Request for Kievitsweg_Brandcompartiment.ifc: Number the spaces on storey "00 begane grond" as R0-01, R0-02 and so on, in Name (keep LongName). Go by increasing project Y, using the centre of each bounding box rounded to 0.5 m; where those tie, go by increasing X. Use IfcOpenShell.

First a look at what the model holds.

```python
import ifcopenshell
import ifcopenshell.util.element
import ifcopenshell.util.placement

model = ifcopenshell.open("Kievitsweg_Brandcompartiment.ifc")
print(model.schema)
storey = next(s for s in model.by_type("IfcBuildingStorey") if s.Name == "00 begane grond")
spaces = [e for e in ifcopenshell.util.element.get_decomposition(storey) if e.is_a("IfcSpace")]
for e in sorted(spaces, key=lambda e: e.id()):
    origin = ifcopenshell.util.placement.get_local_placement(e.ObjectPlacement)[:3, 3]
    print(e.id(), e.Name, e.LongName, origin.round(2) + 0.0, sep=" | ")
```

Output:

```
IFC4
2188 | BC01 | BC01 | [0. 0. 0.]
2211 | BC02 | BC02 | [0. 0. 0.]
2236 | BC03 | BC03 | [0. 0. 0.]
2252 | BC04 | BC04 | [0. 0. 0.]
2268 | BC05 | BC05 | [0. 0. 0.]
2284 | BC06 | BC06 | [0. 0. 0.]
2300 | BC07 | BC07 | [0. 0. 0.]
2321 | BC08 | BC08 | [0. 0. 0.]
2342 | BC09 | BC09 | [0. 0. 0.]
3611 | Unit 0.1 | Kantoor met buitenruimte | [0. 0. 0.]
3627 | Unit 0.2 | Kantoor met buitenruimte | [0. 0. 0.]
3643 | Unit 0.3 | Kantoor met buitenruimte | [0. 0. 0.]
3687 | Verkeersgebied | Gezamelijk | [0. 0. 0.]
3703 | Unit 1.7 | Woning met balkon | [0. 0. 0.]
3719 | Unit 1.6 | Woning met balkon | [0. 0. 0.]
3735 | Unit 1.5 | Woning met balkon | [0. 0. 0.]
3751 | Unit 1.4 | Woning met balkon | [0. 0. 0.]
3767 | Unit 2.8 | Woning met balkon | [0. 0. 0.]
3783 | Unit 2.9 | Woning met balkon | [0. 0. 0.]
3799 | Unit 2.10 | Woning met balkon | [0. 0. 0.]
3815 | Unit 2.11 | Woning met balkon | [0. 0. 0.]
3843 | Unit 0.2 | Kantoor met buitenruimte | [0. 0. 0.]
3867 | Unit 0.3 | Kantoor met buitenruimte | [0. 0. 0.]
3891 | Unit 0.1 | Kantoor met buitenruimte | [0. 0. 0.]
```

```python
import ifcopenshell
import ifcopenshell.geom
import ifcopenshell.util.element
import ifcopenshell.util.shape

model = ifcopenshell.open("Kievitsweg_Brandcompartiment.ifc")
settings = ifcopenshell.geom.settings()
settings.set("use-world-coords", True)


def centre(element):
    shape = ifcopenshell.geom.create_shape(settings, element)
    return ifcopenshell.util.shape.get_bbox_centroid(shape.geometry)


storey = next(s for s in model.by_type("IfcBuildingStorey") if s.Name == "00 begane grond")
spaces = [e for e in ifcopenshell.util.element.get_decomposition(storey) if e.is_a("IfcSpace")]

# Insertion points can sit at a corner or the storey origin, so sort by the geometry (in metres).
centres = {e: centre(e) for e in spaces}
spaces.sort(key=lambda e: (round(centres[e][1] / 0.5), centres[e][0]))

for i, e in enumerate(spaces, start=1):
    number = f"R0-{i:02d}"
    e.Name = number
    print(e.id(), number)

model.write("Kievitsweg_Brandcompartiment_rev.ifc")
```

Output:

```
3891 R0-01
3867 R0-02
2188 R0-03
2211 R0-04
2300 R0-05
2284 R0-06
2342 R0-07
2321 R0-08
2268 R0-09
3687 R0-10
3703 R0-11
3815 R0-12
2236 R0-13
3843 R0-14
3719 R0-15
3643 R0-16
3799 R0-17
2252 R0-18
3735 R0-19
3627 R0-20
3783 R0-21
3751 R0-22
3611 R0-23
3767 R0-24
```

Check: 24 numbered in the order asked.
